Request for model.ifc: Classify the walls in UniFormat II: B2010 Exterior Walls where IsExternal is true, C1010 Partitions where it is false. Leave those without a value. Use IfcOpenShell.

First a look at what the model holds.

```python
import ifcopenshell
import ifcopenshell.util.element

model = ifcopenshell.open("model.ifc")
print(model.schema)
print("classifications:", [c.Name for c in model.by_type("IfcClassification")])
values = [ifcopenshell.util.element.get_pset(e, "Pset_WallCommon", "IsExternal") for e in model.by_type("IfcWall")]
for value in (True, False, None):
    print("IsExternal", value, values.count(value))
```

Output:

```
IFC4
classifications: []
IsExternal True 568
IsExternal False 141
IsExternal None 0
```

```python
import ifcopenshell
import ifcopenshell.api.classification
import ifcopenshell.util.element

model = ifcopenshell.open("model.ifc")

system = ifcopenshell.api.classification.add_classification(model, classification="UniFormat II")

walls = model.by_type("IfcWall")
external = {e: ifcopenshell.util.element.get_pset(e, "Pset_WallCommon", "IsExternal") for e in walls}
for flag, code, name in ((True, "B2010", "Exterior Walls"), (False, "C1010", "Partitions")):
    products = [e for e in walls if external[e] is flag]
    ifcopenshell.api.classification.add_reference(
        model, products=products, classification=system, identification=code, name=name
    )
    print(code, len(products))

model.write("model_rev.ifc")
```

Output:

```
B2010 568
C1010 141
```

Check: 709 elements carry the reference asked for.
